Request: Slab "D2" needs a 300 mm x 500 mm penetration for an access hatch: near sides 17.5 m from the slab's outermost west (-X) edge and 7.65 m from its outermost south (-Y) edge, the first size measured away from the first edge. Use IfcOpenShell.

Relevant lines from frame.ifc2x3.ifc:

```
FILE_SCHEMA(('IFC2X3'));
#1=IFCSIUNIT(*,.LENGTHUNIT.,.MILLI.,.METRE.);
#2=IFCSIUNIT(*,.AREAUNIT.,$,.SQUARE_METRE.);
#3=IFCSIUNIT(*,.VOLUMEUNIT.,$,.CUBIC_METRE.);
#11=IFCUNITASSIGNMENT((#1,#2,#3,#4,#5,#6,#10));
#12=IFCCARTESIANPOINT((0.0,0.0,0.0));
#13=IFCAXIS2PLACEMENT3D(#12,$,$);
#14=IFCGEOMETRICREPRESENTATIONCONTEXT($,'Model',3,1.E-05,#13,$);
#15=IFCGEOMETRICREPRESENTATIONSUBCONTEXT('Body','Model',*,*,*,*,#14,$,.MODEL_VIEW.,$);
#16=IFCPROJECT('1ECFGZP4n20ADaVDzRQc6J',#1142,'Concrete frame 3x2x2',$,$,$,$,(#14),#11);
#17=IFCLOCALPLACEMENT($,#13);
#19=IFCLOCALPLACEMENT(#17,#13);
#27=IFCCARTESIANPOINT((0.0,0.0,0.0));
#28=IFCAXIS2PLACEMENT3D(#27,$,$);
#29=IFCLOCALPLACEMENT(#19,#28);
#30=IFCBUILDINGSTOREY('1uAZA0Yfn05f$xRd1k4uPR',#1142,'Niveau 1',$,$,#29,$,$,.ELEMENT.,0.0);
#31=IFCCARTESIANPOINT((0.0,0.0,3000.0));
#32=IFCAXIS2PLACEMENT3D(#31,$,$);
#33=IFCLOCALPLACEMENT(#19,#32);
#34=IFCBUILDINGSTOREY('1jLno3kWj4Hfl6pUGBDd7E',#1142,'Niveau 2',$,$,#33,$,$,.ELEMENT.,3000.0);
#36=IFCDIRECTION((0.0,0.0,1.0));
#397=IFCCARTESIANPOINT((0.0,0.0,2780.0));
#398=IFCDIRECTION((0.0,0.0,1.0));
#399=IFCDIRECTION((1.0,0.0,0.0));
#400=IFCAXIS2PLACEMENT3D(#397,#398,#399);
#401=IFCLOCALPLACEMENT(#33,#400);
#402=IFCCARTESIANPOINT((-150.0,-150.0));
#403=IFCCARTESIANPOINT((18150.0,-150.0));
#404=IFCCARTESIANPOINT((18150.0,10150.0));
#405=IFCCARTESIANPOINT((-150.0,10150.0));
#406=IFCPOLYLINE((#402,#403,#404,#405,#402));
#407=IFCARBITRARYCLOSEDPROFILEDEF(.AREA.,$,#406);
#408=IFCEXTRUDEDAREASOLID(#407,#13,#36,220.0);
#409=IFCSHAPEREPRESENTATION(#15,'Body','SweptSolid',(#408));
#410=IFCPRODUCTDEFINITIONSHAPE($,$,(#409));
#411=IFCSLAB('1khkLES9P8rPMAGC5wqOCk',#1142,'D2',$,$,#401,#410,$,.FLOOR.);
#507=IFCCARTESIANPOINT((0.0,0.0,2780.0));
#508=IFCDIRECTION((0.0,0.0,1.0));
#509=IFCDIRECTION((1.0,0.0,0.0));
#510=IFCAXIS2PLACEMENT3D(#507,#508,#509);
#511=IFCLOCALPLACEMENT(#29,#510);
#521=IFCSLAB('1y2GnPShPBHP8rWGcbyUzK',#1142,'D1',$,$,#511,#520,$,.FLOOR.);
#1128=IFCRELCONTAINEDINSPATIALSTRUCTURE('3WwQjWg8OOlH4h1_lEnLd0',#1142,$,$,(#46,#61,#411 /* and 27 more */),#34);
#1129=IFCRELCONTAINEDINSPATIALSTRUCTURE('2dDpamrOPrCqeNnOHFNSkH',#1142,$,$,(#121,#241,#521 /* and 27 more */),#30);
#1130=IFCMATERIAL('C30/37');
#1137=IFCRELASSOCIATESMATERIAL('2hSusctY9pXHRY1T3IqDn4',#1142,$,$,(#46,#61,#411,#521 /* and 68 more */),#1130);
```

```python
import numpy as np
import ifcopenshell
import ifcopenshell.api.feature
import ifcopenshell.api.geometry
import ifcopenshell.api.root
import ifcopenshell.geom
import ifcopenshell.util.placement
import ifcopenshell.util.representation
import ifcopenshell.util.shape
import ifcopenshell.util.unit

model = ifcopenshell.open("frame.ifc2x3.ifc")
unit_scale = ifcopenshell.util.unit.calculate_unit_scale(model)
settings = ifcopenshell.geom.settings()


def volume(element):
    """Net volume in cubic metres, openings subtracted."""
    shape = ifcopenshell.geom.create_shape(settings, element)
    return ifcopenshell.util.shape.get_volume(shape.geometry)


slab = model.by_id(411)
before = volume(slab)

# Extent in the slab's own axes, in metres. The edges named are its -X and -Y sides.
slab_shape = ifcopenshell.geom.create_shape(settings, slab)
vertices = ifcopenshell.util.shape.get_vertices(slab_shape.geometry)
x_min, y_min, bottom = vertices.min(axis=0)
top = vertices[:, 2].max()

opening = ifcopenshell.api.root.create_entity(model, ifc_class="IfcOpeningElement", name="Access hatch opening")
context = ifcopenshell.util.representation.get_context(model, "Model", "Body", "MODEL_VIEW")
width, depth = 0.3, 0.5
outline = [(0.0, 0.0), (width, 0.0), (width, depth), (0.0, depth), (0.0, 0.0)]
# Overshoot both faces by 50 mm so the cut is clean.
shape = ifcopenshell.api.geometry.add_slab_representation(
    model, context=context, depth=top - bottom + 0.1, polyline=outline
)
ifcopenshell.api.geometry.assign_representation(model, product=opening, representation=shape)

matrix = ifcopenshell.util.placement.get_local_placement(slab.ObjectPlacement)
matrix[:, 3] = matrix @ np.append(np.array([x_min + 17.5, y_min + 7.65, bottom - 0.05]) / unit_scale, 1.0)
ifcopenshell.api.geometry.edit_object_placement(model, product=opening, matrix=matrix, is_si=False)
ifcopenshell.api.feature.add_feature(model, feature=opening, element=slab)

after = volume(slab)

print(f"slab volume {before:.3f} -> {after:.3f} m3")

model.write("frame.ifc2x3-out.ifc")
```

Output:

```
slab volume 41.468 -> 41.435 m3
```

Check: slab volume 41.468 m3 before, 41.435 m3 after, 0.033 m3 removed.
